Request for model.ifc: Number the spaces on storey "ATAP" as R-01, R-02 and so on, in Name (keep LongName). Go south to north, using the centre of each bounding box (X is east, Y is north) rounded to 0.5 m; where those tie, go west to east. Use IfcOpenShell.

First a look at what the model holds.

```python
import ifcopenshell
import ifcopenshell.util.element
import ifcopenshell.util.placement

model = ifcopenshell.open("model.ifc")
print(model.schema)
storey = next(s for s in model.by_type("IfcBuildingStorey") if s.Name == "ATAP")
spaces = [e for e in ifcopenshell.util.element.get_decomposition(storey) if e.is_a("IfcSpace")]
for e in sorted(spaces, key=lambda e: e.id()):
    origin = ifcopenshell.util.placement.get_local_placement(e.ObjectPlacement)[:3, 3]
    print(e.id(), e.Name, e.LongName, origin.round(2) + 0.0, sep=" | ")
```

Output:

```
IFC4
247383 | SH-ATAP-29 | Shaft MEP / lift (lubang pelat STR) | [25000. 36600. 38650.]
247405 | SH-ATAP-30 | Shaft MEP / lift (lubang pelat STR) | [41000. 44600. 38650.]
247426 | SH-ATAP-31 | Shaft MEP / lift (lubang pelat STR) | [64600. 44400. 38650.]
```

```python
import ifcopenshell
import ifcopenshell.geom
import ifcopenshell.util.element
import ifcopenshell.util.shape

model = ifcopenshell.open("model.ifc")
settings = ifcopenshell.geom.settings()
settings.set("use-world-coords", True)


def centre(element):
    shape = ifcopenshell.geom.create_shape(settings, element)
    return ifcopenshell.util.shape.get_bbox_centroid(shape.geometry)


storey = next(s for s in model.by_type("IfcBuildingStorey") if s.Name == "ATAP")
spaces = [e for e in ifcopenshell.util.element.get_decomposition(storey) if e.is_a("IfcSpace")]

# Insertion points can sit at a corner or the storey origin, so sort by the geometry (in metres).
centres = {e: centre(e) for e in spaces}
spaces.sort(key=lambda e: (round(centres[e][1] / 0.5), centres[e][0]))

for i, e in enumerate(spaces, start=1):
    number = f"R-{i:02d}"
    e.Name = number
    print(e.id(), number)

model.write("model_rev.ifc")
```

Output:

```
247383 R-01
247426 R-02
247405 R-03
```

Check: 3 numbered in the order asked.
